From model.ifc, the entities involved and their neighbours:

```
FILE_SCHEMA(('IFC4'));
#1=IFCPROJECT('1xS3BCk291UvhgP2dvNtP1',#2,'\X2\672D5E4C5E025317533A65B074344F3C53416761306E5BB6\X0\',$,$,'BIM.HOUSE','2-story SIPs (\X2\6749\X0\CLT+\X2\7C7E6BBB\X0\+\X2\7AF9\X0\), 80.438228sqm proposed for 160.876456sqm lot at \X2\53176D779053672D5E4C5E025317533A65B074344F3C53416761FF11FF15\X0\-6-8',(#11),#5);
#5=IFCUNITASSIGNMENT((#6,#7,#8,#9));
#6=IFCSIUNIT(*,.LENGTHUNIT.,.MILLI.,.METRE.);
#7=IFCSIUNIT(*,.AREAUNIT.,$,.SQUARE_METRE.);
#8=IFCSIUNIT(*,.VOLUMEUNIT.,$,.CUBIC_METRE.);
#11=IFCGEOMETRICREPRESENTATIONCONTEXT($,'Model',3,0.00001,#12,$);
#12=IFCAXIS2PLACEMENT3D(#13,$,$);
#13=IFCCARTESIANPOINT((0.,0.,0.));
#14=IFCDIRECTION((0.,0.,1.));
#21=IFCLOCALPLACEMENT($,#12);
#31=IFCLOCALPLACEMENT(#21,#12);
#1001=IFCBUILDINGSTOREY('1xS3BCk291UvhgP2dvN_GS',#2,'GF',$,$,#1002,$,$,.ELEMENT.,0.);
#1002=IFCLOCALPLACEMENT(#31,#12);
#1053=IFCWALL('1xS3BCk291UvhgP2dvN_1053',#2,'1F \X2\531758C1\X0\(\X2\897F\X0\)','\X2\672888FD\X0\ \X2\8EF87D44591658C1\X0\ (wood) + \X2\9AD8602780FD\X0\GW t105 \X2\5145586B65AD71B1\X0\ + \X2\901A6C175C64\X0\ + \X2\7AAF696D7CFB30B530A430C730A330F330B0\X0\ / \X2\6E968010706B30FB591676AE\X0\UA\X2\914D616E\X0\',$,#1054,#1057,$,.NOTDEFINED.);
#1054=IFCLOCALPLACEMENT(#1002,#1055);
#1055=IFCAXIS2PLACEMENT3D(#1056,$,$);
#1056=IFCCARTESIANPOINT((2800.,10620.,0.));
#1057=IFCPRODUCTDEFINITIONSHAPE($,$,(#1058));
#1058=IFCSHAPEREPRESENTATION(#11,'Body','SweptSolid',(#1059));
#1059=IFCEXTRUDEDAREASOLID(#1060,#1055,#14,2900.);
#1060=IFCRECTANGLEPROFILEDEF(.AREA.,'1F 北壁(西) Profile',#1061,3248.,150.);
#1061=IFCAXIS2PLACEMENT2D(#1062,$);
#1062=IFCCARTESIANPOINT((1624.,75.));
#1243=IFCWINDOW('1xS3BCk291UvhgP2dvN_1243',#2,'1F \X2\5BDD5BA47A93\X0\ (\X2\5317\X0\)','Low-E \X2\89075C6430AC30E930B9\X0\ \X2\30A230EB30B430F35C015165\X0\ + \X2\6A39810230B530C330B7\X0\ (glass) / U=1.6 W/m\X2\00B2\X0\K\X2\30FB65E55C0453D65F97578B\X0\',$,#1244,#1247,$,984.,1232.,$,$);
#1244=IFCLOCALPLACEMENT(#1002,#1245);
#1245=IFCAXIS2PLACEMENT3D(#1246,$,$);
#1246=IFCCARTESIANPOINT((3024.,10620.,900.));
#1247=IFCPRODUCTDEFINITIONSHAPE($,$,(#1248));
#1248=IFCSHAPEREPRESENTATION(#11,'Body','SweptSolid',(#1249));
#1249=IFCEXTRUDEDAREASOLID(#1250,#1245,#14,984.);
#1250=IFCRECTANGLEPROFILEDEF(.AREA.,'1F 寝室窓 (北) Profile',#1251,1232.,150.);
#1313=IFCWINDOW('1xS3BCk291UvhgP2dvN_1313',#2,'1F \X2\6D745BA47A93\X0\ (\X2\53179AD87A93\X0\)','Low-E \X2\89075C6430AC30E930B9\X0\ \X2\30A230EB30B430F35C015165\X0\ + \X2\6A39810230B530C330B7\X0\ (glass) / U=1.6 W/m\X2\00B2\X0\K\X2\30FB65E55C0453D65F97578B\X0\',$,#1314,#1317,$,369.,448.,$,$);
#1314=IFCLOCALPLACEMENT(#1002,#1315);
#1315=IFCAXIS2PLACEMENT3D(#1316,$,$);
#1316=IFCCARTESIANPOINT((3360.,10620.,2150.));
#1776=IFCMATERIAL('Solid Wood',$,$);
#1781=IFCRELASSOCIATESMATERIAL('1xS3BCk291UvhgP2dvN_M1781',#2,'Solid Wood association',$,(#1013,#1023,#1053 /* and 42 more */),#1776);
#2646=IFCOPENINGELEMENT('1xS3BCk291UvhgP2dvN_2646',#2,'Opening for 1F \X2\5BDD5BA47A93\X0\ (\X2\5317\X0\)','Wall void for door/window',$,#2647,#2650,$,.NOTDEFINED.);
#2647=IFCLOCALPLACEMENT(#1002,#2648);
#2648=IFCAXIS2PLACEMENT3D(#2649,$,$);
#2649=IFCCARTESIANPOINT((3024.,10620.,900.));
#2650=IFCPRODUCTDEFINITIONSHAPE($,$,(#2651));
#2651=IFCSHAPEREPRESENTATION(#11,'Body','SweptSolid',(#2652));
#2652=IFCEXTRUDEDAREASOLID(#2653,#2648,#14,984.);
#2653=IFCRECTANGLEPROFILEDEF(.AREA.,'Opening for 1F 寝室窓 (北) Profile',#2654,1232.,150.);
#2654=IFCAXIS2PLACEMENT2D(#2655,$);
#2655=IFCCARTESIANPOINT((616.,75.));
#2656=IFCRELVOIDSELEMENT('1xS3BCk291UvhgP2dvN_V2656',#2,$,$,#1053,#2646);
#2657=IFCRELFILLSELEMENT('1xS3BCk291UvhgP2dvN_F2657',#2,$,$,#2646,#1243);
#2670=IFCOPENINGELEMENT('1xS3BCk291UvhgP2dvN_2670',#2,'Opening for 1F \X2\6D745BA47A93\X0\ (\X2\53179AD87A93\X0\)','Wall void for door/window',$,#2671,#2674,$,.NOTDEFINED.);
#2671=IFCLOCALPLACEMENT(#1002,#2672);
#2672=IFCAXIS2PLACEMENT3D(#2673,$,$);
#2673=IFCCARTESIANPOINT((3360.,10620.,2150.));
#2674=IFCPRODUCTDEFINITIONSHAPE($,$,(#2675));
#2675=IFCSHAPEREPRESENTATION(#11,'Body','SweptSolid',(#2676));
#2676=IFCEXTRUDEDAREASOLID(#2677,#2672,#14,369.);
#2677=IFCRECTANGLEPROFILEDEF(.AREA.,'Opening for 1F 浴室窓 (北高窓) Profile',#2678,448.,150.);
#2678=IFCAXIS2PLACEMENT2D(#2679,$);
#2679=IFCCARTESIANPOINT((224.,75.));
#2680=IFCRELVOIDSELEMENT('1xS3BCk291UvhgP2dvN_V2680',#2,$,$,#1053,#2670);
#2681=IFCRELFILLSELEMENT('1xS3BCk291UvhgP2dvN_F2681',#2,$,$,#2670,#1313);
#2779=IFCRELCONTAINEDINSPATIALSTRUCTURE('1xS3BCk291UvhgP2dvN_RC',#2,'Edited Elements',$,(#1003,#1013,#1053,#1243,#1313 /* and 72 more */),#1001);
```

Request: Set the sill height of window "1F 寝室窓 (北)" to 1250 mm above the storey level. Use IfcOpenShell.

```python
import numpy as np
import ifcopenshell
import ifcopenshell.api.geometry
import ifcopenshell.geom
import ifcopenshell.util.element
import ifcopenshell.util.placement
import ifcopenshell.util.shape
import ifcopenshell.util.unit

model = ifcopenshell.open("model.ifc")
unit_scale = ifcopenshell.util.unit.calculate_unit_scale(model)

window = model.by_id(1243)
opening = window.FillsVoids[0].RelatingOpeningElement
storey = ifcopenshell.util.element.get_container(window, ifc_class="IfcBuildingStorey")
level = ifcopenshell.util.placement.get_local_placement(storey.ObjectPlacement)[2, 3]

# The opening's origin need not be at the sill, so measure its lowest point.
shape = ifcopenshell.geom.create_shape(ifcopenshell.geom.settings(), opening)
bottom = ifcopenshell.util.shape.get_shape_bottom_elevation(shape, shape.geometry) / unit_scale
dz = level + 1.25 / unit_scale - bottom

shift = np.array([0.0, 0.0, dz])
# The window is not placed relative to its opening, so move both.
for product in (opening, window):
    matrix = ifcopenshell.util.placement.get_local_placement(product.ObjectPlacement)
    matrix[:3, 3] += shift
    ifcopenshell.api.geometry.edit_object_placement(model, product=product, matrix=matrix, is_si=False)

print(f"moved by {dz * unit_scale:+.3f} m")

model.write("model-out.ifc")
```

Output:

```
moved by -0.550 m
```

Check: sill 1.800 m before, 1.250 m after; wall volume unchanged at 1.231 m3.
